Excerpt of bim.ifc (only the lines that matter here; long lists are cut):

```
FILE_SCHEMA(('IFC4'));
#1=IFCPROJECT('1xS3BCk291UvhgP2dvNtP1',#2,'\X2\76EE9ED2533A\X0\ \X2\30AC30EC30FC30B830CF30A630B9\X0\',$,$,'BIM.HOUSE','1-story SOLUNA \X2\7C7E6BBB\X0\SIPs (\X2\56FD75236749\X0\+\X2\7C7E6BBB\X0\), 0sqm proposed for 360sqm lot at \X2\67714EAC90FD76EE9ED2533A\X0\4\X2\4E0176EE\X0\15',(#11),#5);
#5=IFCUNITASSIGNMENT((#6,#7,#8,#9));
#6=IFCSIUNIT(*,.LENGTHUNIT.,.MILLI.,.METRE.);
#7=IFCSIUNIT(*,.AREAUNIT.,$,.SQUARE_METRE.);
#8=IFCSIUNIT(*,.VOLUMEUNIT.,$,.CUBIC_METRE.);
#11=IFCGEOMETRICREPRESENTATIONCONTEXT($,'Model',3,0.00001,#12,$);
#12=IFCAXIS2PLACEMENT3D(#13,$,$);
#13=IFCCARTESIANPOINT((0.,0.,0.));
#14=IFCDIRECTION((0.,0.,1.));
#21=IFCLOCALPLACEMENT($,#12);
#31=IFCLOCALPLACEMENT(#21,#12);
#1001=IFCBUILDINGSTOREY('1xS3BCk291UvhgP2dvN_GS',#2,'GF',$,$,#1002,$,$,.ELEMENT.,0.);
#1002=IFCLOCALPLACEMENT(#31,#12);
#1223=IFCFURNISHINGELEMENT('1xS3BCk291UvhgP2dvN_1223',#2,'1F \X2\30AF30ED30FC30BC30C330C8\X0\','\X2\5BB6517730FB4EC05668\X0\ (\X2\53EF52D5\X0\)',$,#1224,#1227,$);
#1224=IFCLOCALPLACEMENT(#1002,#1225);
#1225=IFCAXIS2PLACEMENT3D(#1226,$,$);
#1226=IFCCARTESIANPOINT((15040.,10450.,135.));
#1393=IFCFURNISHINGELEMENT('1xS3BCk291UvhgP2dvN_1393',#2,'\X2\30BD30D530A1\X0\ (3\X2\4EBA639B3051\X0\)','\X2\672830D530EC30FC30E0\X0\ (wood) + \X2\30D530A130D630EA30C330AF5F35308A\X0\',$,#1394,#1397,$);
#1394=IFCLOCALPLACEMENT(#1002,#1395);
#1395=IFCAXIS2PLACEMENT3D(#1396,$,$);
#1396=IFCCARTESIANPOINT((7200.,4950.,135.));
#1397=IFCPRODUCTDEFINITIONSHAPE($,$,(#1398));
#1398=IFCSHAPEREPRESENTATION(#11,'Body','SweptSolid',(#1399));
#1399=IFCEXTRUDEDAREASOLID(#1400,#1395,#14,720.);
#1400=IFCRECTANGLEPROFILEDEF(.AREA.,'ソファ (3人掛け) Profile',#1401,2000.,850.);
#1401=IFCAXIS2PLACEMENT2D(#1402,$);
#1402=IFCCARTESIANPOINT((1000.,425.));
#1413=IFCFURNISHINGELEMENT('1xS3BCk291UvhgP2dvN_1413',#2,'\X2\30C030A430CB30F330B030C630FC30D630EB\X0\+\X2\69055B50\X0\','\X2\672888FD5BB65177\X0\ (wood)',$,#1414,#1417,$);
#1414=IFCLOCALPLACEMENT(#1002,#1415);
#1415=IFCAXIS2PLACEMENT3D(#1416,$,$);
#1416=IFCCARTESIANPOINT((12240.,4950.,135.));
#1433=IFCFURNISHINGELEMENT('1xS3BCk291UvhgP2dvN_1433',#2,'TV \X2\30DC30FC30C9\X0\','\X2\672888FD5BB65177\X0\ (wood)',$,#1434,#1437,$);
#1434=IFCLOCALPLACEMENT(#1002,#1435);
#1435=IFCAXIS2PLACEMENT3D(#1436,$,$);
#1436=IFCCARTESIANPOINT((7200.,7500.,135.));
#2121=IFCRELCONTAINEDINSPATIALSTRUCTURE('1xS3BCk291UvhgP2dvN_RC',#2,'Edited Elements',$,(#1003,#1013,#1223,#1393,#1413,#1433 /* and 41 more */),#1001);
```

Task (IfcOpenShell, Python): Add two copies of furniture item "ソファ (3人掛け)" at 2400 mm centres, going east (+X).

```python
import numpy as np
import ifcopenshell
import ifcopenshell.api.geometry
import ifcopenshell.api.root
import ifcopenshell.util.element
import ifcopenshell.util.placement
import ifcopenshell.util.unit

model = ifcopenshell.open("bim.ifc")
unit_scale = ifcopenshell.util.unit.calculate_unit_scale(model)


def reuse_history(source, copy):
    """copy_class also copies each property set's owner history, people and application; keep the originals."""
    for rel in copy.IsDefinedBy:
        if rel.is_a("IfcRelDefinesByProperties") and (history := rel.RelatingPropertyDefinition.OwnerHistory):
            rel.RelatingPropertyDefinition.OwnerHistory = source.OwnerHistory
            ifcopenshell.util.element.remove_deep2(model, history)


source = model.by_guid("1xS3BCk291UvhgP2dvN_1393")
base = ifcopenshell.util.placement.get_local_placement(source.ObjectPlacement)
step = np.array([1.0, 0.0, 0.0]) * 2.4 / unit_scale

for i in range(1, 3):
    copy = ifcopenshell.api.root.copy_class(model, product=source)
    copy.Representation = ifcopenshell.util.element.copy_deep(
        model, source.Representation, exclude=["IfcGeometricRepresentationContext", "IfcRepresentationMap"]
    )
    reuse_history(source, copy)
    matrix = base.copy()
    matrix[:3, 3] += i * step
    print("added at", matrix[:3, 3].round(3) + 0.0)
    ifcopenshell.api.geometry.edit_object_placement(model, product=copy, matrix=matrix, is_si=False)

model.write("bim_edited.ifc")
```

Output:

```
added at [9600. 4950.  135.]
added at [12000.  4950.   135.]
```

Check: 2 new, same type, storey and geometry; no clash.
